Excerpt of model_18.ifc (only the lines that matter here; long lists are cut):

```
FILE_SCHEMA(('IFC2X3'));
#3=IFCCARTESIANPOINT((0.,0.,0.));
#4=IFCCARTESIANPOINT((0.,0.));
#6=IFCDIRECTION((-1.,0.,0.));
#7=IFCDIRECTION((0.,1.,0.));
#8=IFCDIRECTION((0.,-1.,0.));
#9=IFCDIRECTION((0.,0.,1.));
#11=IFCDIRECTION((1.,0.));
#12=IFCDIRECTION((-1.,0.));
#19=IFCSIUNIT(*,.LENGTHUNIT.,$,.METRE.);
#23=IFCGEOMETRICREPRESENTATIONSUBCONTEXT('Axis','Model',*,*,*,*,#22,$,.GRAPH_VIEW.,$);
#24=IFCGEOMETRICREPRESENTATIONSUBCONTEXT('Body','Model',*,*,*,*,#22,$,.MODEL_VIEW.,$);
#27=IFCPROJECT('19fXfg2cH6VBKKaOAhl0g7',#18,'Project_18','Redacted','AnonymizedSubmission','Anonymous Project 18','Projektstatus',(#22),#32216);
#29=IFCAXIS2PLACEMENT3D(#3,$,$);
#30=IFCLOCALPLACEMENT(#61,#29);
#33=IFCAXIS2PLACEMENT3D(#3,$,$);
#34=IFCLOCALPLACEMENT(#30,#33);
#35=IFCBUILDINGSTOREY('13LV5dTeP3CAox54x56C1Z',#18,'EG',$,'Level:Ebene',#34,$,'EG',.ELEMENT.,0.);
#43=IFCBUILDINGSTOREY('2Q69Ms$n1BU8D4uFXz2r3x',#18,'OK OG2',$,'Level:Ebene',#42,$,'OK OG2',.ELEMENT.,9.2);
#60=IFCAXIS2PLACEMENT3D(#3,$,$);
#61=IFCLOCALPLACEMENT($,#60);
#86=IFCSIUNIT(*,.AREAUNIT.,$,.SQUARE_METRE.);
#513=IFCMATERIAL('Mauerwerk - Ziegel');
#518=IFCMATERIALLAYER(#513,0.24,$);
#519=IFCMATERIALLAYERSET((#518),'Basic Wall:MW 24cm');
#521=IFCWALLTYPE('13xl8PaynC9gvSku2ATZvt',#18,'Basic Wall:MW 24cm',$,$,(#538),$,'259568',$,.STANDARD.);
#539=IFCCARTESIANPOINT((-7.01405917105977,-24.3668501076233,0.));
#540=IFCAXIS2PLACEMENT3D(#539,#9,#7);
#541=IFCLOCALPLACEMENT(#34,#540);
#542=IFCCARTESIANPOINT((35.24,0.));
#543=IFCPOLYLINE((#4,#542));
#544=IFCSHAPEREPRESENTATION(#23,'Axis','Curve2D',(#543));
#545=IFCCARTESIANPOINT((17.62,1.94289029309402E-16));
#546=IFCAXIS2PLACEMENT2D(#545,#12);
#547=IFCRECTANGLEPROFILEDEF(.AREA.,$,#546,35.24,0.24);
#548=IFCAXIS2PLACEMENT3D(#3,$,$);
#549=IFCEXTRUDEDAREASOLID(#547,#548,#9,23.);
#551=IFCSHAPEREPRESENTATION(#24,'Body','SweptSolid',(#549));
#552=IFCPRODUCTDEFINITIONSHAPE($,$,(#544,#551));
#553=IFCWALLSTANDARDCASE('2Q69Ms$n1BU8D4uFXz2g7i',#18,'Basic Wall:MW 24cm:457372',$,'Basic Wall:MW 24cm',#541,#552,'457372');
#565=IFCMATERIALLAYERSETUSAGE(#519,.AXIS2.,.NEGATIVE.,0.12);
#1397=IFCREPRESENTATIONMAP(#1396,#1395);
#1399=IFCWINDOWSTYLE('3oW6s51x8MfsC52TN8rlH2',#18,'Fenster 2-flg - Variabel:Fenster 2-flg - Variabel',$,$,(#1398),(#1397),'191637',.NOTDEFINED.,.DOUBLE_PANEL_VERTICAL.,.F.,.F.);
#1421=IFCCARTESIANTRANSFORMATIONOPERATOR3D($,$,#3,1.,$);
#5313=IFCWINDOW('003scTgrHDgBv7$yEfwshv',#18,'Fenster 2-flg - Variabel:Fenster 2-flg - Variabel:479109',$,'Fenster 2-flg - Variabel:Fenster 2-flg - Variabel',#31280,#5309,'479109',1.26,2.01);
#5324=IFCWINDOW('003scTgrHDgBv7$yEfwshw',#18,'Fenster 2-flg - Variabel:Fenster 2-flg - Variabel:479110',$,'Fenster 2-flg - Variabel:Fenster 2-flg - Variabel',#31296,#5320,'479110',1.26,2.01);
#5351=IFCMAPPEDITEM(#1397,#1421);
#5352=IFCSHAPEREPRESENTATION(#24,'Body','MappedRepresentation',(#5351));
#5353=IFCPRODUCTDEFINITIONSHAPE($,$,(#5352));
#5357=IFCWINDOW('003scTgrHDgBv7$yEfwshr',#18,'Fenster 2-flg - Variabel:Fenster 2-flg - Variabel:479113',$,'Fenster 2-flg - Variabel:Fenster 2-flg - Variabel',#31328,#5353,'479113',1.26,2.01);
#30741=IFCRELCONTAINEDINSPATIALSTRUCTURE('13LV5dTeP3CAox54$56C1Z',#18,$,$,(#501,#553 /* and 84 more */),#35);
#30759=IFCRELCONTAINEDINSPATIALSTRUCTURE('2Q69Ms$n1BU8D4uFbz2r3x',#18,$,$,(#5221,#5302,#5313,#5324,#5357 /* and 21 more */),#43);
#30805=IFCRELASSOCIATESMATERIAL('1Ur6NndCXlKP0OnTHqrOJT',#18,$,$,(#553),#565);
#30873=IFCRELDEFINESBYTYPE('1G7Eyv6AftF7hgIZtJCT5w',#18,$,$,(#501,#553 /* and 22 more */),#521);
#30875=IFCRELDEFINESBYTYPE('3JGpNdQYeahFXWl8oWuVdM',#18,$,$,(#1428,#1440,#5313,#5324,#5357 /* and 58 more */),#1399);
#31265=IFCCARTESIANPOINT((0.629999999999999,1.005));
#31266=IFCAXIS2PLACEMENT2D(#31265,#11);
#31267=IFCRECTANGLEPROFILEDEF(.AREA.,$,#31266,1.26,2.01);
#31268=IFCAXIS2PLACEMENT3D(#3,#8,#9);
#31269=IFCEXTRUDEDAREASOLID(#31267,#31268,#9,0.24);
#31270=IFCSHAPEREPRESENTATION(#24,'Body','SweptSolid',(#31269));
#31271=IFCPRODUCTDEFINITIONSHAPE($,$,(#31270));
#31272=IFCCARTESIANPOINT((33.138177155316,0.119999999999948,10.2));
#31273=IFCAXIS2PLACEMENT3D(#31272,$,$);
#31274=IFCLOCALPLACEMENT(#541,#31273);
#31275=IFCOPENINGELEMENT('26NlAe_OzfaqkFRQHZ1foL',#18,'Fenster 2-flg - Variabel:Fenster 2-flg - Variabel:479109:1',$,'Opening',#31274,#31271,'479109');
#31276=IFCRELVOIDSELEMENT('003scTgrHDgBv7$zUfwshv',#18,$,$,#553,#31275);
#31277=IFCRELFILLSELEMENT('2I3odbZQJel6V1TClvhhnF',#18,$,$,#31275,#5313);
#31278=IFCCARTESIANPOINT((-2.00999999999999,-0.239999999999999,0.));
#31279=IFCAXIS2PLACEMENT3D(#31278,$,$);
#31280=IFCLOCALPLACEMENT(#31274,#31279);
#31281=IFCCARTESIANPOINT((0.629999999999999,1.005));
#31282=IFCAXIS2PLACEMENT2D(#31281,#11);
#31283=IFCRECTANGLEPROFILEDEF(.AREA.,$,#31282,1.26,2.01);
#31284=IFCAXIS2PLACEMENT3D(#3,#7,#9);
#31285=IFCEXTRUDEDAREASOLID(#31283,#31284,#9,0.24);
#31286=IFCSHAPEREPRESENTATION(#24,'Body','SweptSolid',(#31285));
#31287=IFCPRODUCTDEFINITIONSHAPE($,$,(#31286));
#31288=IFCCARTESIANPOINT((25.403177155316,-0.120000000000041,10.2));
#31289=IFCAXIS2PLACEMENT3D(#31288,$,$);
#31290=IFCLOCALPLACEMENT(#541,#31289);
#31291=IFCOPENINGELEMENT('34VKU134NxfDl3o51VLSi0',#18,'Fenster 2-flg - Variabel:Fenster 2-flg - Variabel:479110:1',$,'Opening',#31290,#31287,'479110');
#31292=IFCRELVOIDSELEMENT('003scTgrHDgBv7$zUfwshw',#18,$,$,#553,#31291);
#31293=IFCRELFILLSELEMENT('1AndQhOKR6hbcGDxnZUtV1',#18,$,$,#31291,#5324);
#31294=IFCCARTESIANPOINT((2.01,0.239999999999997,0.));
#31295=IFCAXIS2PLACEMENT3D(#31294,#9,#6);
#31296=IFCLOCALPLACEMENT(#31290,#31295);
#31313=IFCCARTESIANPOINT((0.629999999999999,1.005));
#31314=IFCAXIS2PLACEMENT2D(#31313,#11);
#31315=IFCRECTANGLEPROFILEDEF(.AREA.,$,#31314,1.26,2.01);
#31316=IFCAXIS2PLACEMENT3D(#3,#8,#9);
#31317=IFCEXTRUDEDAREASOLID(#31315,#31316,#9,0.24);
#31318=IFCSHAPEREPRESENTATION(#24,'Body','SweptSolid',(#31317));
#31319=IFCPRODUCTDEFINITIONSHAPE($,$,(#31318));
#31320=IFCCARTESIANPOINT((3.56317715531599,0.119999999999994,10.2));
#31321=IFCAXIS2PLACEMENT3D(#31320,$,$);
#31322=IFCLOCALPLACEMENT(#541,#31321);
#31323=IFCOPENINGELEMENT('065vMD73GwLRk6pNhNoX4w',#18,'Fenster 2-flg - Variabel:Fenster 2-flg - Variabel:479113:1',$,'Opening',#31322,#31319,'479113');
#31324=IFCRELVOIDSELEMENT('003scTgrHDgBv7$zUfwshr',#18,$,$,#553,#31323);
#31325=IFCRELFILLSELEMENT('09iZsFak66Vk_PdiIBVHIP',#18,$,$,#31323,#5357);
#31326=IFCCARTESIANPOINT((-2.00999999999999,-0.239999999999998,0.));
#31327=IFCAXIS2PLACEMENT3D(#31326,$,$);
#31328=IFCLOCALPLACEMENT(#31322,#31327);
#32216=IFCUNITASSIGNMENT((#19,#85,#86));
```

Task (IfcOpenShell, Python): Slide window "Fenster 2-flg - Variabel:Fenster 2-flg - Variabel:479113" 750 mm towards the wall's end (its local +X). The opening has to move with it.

```python
import ifcopenshell
import ifcopenshell.api.geometry
import ifcopenshell.util.placement

model = ifcopenshell.open("model_18.ifc")

window = model.by_id(5357)
opening = window.FillsVoids[0].RelatingOpeningElement
wall = opening.VoidsElements[0].RelatingBuildingElement

wall_matrix = ifcopenshell.util.placement.get_local_placement(wall.ObjectPlacement)
shift = wall_matrix[:3, 0] * 0.75
before = ifcopenshell.util.placement.get_local_placement(window.ObjectPlacement)[:3, 3].copy()

# The window is placed relative to its opening, so it follows when the opening moves.
matrix = ifcopenshell.util.placement.get_local_placement(opening.ObjectPlacement)
matrix[:3, 3] += shift
ifcopenshell.api.geometry.edit_object_placement(
    model, product=opening, matrix=matrix, is_si=False, should_transform_children=True
)

after = ifcopenshell.util.placement.get_local_placement(window.ObjectPlacement)[:3, 3]
print("window moved by", (after - before).round(3) + 0.0)

model.write("model_18_edited.ifc")
```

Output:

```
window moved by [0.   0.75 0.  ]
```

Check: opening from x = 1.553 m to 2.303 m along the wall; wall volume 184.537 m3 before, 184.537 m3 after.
